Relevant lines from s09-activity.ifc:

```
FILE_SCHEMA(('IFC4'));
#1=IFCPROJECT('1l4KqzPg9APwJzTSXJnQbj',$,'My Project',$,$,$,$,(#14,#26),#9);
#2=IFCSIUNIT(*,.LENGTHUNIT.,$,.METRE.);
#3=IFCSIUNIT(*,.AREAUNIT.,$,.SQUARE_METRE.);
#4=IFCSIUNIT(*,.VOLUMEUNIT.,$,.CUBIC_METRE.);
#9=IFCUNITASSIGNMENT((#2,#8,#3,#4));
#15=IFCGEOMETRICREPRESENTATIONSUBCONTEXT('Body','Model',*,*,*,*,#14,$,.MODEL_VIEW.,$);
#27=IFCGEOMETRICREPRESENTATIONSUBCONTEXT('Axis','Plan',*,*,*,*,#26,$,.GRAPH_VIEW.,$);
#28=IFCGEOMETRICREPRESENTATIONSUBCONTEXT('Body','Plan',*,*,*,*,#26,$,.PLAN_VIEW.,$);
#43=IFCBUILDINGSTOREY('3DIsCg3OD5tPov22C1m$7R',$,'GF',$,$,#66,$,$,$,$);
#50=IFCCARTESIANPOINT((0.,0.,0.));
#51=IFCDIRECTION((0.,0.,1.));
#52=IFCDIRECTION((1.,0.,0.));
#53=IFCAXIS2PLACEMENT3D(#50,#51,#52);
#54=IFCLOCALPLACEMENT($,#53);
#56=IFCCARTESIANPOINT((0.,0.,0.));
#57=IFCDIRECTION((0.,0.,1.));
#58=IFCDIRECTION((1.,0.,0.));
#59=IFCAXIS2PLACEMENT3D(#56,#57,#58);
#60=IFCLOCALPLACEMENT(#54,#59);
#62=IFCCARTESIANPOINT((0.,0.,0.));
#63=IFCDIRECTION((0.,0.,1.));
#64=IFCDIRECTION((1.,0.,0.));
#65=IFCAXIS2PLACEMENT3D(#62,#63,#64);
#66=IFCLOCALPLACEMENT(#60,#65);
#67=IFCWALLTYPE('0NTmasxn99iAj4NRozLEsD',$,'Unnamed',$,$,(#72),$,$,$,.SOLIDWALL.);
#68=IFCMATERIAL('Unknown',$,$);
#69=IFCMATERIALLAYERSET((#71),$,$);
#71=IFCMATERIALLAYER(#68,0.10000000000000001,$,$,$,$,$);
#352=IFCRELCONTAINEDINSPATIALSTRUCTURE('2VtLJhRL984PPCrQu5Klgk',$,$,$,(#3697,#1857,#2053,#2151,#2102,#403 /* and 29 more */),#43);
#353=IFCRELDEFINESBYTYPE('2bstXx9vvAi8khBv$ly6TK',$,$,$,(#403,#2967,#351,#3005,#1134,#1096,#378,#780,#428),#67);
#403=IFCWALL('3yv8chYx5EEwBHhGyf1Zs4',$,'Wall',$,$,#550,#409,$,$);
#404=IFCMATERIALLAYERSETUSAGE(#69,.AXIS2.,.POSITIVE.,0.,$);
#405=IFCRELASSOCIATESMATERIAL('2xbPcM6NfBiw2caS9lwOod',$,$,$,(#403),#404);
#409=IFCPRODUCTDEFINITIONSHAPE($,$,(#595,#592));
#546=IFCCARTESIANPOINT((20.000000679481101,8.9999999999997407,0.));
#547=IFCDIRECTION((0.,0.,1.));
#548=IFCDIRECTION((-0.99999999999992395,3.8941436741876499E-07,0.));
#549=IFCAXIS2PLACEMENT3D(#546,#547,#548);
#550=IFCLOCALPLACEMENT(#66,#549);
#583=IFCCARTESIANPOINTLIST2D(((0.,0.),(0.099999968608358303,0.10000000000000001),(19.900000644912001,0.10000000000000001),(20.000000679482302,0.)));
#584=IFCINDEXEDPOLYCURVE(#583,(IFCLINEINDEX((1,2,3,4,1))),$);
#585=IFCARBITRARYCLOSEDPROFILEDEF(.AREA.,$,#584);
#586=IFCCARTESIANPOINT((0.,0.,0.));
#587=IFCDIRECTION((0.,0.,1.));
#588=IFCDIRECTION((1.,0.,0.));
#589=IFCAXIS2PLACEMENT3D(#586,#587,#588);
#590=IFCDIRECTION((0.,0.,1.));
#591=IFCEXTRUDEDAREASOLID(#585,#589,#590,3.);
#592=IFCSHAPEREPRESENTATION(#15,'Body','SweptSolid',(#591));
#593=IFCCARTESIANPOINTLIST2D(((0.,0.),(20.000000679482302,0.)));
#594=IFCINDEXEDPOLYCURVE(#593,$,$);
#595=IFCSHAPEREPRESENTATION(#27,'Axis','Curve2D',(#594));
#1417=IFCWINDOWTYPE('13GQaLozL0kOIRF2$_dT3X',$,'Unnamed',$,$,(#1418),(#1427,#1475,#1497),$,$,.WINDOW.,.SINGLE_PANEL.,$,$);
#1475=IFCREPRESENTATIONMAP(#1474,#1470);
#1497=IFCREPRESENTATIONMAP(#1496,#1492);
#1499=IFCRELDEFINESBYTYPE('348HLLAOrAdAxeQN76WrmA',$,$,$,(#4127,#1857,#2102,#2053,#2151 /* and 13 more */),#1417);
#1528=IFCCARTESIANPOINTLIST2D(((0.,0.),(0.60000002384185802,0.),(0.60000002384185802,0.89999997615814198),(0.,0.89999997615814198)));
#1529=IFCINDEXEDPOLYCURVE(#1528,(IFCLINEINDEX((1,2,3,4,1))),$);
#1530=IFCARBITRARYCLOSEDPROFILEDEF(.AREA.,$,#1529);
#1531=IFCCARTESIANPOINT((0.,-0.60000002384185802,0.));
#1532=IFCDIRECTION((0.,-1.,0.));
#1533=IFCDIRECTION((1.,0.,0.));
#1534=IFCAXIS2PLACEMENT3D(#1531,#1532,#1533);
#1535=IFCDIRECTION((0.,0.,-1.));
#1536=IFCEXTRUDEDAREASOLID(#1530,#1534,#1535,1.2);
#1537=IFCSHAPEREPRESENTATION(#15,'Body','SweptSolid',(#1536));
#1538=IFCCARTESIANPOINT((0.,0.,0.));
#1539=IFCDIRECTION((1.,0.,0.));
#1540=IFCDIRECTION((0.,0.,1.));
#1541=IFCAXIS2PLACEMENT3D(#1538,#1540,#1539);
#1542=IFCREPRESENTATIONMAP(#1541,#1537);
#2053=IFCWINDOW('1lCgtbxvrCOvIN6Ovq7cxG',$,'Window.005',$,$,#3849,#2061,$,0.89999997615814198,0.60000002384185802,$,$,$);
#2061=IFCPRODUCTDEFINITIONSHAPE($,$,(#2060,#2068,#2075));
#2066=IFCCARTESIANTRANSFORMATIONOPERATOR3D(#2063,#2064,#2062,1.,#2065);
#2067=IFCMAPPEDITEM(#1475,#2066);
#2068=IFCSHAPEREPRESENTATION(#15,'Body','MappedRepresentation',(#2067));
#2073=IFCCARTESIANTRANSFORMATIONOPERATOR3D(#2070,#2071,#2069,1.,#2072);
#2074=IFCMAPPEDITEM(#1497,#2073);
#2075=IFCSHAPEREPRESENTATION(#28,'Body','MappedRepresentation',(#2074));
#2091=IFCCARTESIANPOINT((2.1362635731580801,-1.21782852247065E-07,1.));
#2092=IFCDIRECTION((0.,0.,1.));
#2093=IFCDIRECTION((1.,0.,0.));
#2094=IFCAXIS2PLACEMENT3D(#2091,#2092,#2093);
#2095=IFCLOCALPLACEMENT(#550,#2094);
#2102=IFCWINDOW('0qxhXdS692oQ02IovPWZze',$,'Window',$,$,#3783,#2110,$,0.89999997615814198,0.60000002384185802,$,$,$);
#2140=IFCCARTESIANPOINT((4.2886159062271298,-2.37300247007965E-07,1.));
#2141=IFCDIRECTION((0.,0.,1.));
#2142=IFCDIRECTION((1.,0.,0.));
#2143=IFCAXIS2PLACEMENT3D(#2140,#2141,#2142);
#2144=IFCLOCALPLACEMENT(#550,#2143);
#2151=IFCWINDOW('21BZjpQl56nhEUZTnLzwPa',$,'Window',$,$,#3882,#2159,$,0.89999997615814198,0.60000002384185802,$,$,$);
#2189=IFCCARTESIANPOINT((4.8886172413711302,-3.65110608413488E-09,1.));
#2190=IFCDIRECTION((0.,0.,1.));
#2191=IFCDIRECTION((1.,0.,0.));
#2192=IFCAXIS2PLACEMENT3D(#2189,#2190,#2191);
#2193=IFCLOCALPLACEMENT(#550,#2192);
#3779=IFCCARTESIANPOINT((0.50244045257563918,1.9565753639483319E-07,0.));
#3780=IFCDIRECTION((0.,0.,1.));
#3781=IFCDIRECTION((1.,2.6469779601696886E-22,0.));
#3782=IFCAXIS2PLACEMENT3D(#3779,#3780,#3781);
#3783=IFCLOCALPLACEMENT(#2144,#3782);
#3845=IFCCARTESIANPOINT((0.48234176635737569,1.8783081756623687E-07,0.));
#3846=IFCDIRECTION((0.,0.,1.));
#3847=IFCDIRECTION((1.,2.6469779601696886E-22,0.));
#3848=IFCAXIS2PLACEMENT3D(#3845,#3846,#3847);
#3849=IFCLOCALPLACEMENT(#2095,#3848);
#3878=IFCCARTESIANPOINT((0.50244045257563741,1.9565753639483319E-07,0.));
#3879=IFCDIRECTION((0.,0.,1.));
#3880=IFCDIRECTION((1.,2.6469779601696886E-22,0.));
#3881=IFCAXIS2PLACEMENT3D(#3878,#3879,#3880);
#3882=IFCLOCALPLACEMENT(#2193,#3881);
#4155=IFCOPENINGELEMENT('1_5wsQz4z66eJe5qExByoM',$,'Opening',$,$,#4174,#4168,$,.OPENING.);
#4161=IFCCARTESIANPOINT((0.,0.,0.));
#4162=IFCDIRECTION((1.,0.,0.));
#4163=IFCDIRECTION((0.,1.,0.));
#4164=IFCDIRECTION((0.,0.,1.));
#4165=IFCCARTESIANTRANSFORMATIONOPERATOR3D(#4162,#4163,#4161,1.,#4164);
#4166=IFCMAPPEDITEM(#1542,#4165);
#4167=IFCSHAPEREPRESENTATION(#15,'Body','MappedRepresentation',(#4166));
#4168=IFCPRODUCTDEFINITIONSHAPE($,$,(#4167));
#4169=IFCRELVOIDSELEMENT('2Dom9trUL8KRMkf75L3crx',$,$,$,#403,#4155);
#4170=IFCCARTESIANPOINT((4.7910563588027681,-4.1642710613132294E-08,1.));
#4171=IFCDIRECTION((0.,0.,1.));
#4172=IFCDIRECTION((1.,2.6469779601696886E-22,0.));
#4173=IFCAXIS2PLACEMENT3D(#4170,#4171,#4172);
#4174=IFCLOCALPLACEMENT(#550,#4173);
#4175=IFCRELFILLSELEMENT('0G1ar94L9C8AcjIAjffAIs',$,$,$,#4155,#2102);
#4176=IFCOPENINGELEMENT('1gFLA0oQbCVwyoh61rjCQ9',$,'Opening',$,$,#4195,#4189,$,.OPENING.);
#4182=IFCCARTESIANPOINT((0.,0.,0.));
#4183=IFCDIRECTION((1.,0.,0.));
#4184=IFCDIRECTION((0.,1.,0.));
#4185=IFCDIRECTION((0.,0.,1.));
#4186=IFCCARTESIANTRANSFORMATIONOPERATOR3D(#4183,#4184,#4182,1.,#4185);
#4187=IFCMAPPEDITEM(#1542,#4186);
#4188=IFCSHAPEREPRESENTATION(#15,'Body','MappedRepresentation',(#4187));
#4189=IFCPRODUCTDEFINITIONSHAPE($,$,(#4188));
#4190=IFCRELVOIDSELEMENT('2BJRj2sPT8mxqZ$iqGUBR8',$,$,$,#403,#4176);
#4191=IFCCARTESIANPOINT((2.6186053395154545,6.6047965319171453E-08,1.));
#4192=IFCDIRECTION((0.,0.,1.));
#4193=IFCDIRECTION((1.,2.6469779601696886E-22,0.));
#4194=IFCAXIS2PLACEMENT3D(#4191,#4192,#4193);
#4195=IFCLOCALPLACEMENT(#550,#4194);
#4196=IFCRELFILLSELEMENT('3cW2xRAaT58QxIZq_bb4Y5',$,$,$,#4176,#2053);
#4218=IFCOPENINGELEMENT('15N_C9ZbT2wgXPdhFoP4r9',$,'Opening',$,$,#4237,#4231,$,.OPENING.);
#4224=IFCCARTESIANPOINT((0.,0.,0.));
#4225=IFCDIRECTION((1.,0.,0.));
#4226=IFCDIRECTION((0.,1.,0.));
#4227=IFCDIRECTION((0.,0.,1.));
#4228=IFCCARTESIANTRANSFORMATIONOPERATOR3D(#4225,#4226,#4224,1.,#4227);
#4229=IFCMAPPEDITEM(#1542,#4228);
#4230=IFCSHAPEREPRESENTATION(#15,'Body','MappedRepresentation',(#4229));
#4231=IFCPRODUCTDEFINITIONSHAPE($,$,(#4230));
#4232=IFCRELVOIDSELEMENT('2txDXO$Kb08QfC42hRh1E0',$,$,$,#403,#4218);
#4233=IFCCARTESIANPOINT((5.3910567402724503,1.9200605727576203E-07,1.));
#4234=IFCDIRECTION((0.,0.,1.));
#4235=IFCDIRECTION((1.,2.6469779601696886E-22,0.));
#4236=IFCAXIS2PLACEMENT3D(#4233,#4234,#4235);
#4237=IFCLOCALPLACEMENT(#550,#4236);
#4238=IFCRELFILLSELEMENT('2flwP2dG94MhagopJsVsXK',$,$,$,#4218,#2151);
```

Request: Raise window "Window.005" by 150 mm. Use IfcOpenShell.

```python
import numpy as np
import ifcopenshell
import ifcopenshell.api.geometry
import ifcopenshell.util.placement
import ifcopenshell.util.unit

model = ifcopenshell.open("s09-activity.ifc")
unit_scale = ifcopenshell.util.unit.calculate_unit_scale(model)

window = model.by_guid("1lCgtbxvrCOvIN6Ovq7cxG")
opening = window.FillsVoids[0].RelatingOpeningElement
dz = 0.15 / unit_scale

shift = np.array([0.0, 0.0, dz])
# The window is not placed relative to its opening, so move both.
for product in (opening, window):
    matrix = ifcopenshell.util.placement.get_local_placement(product.ObjectPlacement)
    matrix[:3, 3] += shift
    ifcopenshell.api.geometry.edit_object_placement(model, product=product, matrix=matrix, is_si=False)

print(f"moved by {dz * unit_scale:+.3f} m")

model.write("s09-activity_edited.ifc")
```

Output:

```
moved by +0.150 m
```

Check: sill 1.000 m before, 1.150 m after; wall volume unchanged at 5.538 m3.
